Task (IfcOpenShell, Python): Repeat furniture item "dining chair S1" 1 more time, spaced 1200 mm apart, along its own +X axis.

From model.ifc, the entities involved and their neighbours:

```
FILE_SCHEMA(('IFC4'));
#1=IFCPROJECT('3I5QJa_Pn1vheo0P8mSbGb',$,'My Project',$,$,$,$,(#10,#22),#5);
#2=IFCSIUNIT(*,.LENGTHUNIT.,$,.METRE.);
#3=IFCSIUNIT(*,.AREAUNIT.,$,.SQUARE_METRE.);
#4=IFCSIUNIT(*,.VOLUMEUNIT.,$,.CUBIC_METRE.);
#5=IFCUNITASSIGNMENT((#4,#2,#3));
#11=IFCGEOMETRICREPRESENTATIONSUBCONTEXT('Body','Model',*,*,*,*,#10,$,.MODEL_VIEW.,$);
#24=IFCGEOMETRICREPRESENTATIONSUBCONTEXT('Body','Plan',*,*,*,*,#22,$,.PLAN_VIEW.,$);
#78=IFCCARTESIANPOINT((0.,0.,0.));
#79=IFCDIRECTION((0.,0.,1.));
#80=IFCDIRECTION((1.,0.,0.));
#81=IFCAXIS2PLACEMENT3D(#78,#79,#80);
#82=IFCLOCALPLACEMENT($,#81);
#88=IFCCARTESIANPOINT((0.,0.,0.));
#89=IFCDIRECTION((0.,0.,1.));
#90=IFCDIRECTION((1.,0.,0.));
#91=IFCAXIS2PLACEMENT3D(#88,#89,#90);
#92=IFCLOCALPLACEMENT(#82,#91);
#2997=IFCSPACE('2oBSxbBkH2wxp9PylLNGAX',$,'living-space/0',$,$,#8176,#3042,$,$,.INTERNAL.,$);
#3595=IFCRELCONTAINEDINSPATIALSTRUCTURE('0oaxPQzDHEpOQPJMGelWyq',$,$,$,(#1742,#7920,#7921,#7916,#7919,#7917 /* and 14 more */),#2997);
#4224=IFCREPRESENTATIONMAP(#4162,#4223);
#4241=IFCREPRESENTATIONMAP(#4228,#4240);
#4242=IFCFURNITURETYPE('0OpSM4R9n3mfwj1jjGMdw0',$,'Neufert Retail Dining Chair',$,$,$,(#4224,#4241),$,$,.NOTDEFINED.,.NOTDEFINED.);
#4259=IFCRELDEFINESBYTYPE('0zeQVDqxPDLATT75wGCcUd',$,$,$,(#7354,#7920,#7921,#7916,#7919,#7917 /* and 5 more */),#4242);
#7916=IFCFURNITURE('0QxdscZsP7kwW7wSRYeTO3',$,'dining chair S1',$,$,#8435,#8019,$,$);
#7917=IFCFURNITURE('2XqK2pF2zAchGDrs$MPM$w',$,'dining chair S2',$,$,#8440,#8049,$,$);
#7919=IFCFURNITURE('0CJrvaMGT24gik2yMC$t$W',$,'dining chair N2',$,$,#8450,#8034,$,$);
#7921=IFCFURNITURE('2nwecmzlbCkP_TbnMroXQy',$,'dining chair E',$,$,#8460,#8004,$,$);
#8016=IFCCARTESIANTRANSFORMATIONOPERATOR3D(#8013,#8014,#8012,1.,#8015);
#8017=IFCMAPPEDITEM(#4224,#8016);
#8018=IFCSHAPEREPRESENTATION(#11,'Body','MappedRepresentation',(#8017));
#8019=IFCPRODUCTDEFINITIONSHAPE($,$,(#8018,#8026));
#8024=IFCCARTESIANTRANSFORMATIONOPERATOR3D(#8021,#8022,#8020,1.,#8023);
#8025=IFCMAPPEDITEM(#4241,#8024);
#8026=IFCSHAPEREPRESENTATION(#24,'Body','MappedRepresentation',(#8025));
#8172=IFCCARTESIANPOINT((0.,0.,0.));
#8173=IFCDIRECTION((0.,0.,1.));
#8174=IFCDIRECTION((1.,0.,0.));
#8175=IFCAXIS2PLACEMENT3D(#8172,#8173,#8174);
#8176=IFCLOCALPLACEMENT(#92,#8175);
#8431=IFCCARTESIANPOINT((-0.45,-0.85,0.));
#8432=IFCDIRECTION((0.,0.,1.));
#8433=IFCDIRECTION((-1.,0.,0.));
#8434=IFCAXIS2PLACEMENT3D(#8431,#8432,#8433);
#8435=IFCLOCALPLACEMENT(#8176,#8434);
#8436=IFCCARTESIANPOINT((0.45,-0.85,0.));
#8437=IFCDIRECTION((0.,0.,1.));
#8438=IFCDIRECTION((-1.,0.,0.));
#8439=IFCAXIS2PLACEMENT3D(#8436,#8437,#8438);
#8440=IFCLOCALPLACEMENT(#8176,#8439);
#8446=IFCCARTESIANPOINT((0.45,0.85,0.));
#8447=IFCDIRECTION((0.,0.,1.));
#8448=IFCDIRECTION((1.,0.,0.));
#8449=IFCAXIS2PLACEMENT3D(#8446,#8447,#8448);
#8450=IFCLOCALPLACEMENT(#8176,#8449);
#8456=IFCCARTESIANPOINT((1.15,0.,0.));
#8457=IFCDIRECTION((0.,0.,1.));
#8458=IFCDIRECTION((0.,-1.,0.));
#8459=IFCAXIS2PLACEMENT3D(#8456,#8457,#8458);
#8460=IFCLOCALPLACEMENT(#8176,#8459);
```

```python
import ifcopenshell
import ifcopenshell.api.geometry
import ifcopenshell.api.root
import ifcopenshell.util.element
import ifcopenshell.util.placement
import ifcopenshell.util.unit

model = ifcopenshell.open("model.ifc")
unit_scale = ifcopenshell.util.unit.calculate_unit_scale(model)

source = model.by_guid("0QxdscZsP7kwW7wSRYeTO3")
base = ifcopenshell.util.placement.get_local_placement(source.ObjectPlacement)
step = base[:3, 0] * 1.2 / unit_scale

for i in range(1, 2):
    copy = ifcopenshell.api.root.copy_class(model, product=source)
    copy.Representation = ifcopenshell.util.element.copy_deep(
        model, source.Representation, exclude=["IfcGeometricRepresentationContext", "IfcRepresentationMap"]
    )
    matrix = base.copy()
    matrix[:3, 3] += i * step
    print("added at", matrix[:3, 3].round(3) + 0.0)
    ifcopenshell.api.geometry.edit_object_placement(model, product=copy, matrix=matrix, is_si=False)

model.write("model-out.ifc")
```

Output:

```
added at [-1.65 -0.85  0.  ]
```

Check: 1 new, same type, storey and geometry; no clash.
